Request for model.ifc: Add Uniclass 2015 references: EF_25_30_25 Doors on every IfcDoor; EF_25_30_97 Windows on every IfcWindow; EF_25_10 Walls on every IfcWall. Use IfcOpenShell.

First a look at what the model holds.

```python
import ifcopenshell

model = ifcopenshell.open("model.ifc")
print(model.schema)
print("classifications:", [c.Name for c in model.by_type("IfcClassification")])
for ifc_class in ("IfcDoor", "IfcRoof", "IfcStair", "IfcWall", "IfcWindow"):
    print(ifc_class, len(model.by_type(ifc_class)))
```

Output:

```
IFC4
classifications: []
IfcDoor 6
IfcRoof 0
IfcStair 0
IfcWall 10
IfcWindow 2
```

```python
import ifcopenshell
import ifcopenshell.api.classification

model = ifcopenshell.open("model.ifc")

system = ifcopenshell.api.classification.add_classification(model, classification="Uniclass 2015")

codes = {
    "IfcDoor": ("EF_25_30_25", "Doors"),
    "IfcWindow": ("EF_25_30_97", "Windows"),
    "IfcWall": ("EF_25_10", "Walls"),
}
for ifc_class, (code, name) in codes.items():
    products = model.by_type(ifc_class)
    ifcopenshell.api.classification.add_reference(
        model, products=products, classification=system, identification=code, name=name
    )
    print(code, len(products))

model.write("model_edited.ifc")
```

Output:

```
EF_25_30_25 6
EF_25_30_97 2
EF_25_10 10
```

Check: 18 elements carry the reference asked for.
